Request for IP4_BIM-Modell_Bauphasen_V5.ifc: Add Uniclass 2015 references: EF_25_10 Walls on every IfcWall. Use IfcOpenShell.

First a look at what the model holds.

```python
import ifcopenshell

model = ifcopenshell.open("IP4_BIM-Modell_Bauphasen_V5.ifc")
print(model.schema)
print("classifications:", [c.Name for c in model.by_type("IfcClassification")])
for ifc_class in ("IfcDoor", "IfcRoof", "IfcStair", "IfcWall", "IfcWindow"):
    print(ifc_class, len(model.by_type(ifc_class)))
```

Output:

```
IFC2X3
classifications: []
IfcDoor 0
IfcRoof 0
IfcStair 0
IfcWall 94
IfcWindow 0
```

```python
import ifcopenshell
import ifcopenshell.api.classification

model = ifcopenshell.open("IP4_BIM-Modell_Bauphasen_V5.ifc")

# IFC2X3 requires Source and Edition and has no link from the project to the system.
system = model.create_entity("IfcClassification", Source="NBS", Edition="2015", Name="Uniclass 2015")

codes = {
    "IfcWall": ("EF_25_10", "Walls"),
}
for ifc_class, (code, name) in codes.items():
    products = model.by_type(ifc_class)
    ifcopenshell.api.classification.add_reference(
        model, products=products, classification=system, identification=code, name=name
    )
    print(code, len(products))

model.write("IP4_BIM-Modell_Bauphasen_V5_v2.ifc")
```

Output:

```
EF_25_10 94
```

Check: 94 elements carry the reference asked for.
